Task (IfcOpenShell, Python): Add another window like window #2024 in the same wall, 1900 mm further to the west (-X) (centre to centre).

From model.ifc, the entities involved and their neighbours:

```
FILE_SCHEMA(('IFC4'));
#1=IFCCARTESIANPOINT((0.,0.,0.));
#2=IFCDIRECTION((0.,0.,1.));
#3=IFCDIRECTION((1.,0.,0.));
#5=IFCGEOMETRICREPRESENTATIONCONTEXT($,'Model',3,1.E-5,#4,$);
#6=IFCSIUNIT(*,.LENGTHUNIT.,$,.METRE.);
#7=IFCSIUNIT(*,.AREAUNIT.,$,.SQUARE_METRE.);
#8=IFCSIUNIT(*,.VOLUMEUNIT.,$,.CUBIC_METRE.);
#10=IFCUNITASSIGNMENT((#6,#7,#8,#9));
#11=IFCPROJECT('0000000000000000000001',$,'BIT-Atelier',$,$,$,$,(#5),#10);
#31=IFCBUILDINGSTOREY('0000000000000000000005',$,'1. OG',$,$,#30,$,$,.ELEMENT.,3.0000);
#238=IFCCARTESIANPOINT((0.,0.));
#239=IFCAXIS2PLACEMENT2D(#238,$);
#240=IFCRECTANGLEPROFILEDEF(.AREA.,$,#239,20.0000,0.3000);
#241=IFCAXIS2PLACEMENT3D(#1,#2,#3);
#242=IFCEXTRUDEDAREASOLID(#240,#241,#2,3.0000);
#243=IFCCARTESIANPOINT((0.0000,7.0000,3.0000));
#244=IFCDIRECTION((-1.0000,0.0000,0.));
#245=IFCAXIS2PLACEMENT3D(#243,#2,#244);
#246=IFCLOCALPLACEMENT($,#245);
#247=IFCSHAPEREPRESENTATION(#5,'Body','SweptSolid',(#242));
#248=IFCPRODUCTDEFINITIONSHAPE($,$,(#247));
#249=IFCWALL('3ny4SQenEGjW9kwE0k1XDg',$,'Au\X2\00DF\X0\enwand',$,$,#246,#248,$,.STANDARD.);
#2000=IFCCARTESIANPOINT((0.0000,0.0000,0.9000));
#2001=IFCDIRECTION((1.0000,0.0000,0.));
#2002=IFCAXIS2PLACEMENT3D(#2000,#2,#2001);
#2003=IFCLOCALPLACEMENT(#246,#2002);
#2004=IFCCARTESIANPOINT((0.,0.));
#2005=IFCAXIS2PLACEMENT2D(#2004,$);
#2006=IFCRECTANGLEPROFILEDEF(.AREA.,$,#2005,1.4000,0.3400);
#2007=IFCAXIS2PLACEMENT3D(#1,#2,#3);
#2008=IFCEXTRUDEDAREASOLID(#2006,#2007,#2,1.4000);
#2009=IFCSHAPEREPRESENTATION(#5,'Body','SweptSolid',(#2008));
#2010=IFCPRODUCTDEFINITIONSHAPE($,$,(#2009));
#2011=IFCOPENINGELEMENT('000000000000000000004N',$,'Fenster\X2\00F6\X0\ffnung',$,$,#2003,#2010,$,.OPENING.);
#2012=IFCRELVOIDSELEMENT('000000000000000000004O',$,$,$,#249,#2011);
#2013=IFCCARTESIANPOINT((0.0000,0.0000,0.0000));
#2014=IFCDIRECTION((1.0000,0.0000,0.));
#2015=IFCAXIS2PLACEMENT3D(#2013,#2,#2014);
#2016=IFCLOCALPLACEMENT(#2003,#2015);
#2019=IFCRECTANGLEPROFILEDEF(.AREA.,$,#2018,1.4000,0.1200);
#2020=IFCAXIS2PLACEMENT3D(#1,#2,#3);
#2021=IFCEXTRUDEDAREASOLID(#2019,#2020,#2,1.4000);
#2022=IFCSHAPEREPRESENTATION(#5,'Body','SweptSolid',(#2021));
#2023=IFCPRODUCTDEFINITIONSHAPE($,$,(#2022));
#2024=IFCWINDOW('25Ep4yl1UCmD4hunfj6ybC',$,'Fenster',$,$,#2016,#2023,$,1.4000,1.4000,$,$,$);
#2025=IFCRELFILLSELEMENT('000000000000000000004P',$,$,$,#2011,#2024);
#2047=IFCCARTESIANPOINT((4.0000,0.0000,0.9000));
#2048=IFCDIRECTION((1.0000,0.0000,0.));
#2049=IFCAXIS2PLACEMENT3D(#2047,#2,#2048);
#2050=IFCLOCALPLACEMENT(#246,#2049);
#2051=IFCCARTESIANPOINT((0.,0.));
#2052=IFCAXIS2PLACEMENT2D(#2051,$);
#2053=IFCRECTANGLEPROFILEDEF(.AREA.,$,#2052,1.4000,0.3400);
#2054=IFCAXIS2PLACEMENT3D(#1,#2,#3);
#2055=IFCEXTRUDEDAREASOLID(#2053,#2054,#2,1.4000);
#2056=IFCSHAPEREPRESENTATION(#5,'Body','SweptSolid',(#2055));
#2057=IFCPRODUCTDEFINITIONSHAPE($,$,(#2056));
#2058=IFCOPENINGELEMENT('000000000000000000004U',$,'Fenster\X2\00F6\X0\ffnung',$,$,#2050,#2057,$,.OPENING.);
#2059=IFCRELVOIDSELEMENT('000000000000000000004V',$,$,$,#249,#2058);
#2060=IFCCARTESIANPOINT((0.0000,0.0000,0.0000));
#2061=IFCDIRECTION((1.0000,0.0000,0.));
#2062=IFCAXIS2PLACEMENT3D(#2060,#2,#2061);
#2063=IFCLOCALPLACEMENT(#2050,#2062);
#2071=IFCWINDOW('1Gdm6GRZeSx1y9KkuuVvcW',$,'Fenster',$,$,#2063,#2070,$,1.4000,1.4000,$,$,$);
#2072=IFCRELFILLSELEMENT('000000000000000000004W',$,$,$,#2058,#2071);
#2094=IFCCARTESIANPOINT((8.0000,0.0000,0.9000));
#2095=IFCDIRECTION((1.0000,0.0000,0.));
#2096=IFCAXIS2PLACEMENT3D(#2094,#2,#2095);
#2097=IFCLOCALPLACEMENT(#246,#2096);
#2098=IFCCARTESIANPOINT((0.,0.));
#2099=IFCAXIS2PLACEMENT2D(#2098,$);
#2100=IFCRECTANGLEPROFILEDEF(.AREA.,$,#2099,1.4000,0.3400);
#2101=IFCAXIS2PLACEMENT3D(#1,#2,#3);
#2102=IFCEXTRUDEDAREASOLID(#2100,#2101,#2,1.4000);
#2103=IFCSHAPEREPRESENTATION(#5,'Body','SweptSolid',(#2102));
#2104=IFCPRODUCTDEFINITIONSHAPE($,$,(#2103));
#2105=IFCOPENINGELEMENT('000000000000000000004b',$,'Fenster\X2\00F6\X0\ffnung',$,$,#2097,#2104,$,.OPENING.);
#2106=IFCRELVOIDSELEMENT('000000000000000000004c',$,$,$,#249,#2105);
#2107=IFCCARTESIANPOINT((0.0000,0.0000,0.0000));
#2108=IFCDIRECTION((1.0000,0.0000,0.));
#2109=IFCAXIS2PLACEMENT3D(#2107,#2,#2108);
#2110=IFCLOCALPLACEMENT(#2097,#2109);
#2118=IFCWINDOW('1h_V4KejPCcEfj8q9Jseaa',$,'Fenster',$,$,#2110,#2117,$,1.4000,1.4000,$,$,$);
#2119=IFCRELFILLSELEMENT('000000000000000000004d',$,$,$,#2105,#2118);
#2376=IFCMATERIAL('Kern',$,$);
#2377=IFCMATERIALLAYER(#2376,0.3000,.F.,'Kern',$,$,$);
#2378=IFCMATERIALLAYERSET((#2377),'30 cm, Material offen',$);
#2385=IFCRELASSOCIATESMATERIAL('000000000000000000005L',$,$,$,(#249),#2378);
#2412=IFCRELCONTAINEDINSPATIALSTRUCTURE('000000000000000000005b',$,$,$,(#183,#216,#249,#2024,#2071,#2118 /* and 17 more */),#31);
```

```python
import ifcopenshell
import ifcopenshell.api.feature
import ifcopenshell.api.geometry
import ifcopenshell.api.root
import ifcopenshell.geom
import ifcopenshell.util.element
import ifcopenshell.util.placement
import ifcopenshell.util.shape

model = ifcopenshell.open("model.ifc")
settings = ifcopenshell.geom.settings()


def volume(element):
    """Net volume in cubic metres, openings subtracted."""
    shape = ifcopenshell.geom.create_shape(settings, element)
    return ifcopenshell.util.shape.get_volume(shape.geometry)


window = model.by_guid("25Ep4yl1UCmD4hunfj6ybC")
opening = window.FillsVoids[0].RelatingOpeningElement
wall = opening.VoidsElements[0].RelatingBuildingElement
before = volume(wall)
shift = ifcopenshell.util.placement.get_local_placement(wall.ObjectPlacement)[:3, 0] * 1.9

# copy_class copies the void relationship, type, container and properties, but no geometry.
new_opening = ifcopenshell.api.root.copy_class(model, product=opening)
new_opening.Representation = ifcopenshell.util.element.copy_deep(
    model, opening.Representation, exclude=["IfcGeometricRepresentationContext", "IfcRepresentationMap"]
)
new_window = ifcopenshell.api.root.copy_class(model, product=window)
new_window.Representation = ifcopenshell.util.element.copy_deep(
    model, window.Representation, exclude=["IfcGeometricRepresentationContext", "IfcRepresentationMap"]
)
ifcopenshell.api.feature.add_filling(model, opening=new_opening, element=new_window)

for old, new in ((opening, new_opening), (window, new_window)):
    matrix = ifcopenshell.util.placement.get_local_placement(old.ObjectPlacement)
    matrix[:3, 3] += shift
    ifcopenshell.api.geometry.edit_object_placement(model, product=new, matrix=matrix, is_si=False)

after = volume(wall)

print(f"wall volume {before:.3f} -> {after:.3f} m3")

model.write("model_edited.ifc")
```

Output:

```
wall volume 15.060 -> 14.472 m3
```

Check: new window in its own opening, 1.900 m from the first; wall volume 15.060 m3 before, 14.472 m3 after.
